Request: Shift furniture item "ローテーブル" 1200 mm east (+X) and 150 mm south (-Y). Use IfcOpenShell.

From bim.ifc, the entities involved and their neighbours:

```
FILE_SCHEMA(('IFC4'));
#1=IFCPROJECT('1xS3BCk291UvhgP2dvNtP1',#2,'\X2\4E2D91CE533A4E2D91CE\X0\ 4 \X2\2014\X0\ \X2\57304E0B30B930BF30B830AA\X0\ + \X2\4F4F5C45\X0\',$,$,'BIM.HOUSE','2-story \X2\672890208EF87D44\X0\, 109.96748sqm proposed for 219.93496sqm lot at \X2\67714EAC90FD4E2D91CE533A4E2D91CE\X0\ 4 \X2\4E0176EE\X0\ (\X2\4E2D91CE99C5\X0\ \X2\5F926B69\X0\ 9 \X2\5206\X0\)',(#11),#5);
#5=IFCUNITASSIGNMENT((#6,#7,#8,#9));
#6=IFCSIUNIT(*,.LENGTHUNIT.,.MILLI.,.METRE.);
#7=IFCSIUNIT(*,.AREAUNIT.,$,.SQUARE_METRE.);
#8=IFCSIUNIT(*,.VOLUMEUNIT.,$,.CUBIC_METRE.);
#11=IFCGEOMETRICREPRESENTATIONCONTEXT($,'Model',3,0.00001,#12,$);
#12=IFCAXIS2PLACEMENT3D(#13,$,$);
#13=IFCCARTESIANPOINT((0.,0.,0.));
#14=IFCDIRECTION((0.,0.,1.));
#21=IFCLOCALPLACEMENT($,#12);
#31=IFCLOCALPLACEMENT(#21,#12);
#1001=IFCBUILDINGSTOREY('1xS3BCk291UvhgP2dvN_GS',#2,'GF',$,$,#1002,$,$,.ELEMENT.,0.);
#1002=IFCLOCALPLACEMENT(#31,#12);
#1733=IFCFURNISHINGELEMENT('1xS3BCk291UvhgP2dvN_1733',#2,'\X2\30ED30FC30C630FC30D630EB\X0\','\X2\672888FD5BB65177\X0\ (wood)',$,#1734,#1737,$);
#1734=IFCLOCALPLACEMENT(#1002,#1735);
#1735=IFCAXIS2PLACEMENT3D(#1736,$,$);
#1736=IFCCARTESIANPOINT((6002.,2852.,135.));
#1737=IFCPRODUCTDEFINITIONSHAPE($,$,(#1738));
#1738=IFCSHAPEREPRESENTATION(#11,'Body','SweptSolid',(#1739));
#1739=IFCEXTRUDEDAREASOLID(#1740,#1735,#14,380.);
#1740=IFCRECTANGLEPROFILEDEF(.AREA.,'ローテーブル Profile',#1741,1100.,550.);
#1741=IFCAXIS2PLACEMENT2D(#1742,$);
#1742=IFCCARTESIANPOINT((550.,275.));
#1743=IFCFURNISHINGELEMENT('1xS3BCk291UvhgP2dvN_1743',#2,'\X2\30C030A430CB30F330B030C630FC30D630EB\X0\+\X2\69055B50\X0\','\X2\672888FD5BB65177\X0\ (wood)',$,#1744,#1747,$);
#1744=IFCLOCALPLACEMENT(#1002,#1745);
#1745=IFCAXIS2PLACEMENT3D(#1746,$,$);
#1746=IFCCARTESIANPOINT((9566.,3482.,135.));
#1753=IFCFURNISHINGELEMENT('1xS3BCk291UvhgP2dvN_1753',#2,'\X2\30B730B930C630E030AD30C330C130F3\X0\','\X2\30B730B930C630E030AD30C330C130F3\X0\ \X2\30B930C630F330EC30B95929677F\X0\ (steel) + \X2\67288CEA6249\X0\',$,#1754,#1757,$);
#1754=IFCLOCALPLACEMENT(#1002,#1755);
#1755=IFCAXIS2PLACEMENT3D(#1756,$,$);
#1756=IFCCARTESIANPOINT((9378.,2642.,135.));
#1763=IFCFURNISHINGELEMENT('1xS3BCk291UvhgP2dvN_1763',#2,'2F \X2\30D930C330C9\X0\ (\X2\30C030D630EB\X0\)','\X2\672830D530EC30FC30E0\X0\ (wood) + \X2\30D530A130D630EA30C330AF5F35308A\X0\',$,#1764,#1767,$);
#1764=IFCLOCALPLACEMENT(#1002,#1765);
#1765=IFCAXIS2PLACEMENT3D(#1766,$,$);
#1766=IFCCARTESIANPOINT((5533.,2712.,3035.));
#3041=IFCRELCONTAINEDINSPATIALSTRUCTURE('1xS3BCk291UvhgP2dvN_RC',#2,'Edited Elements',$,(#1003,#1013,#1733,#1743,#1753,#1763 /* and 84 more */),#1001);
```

```python
import ifcopenshell
import ifcopenshell.api.geometry
import ifcopenshell.util.placement
import ifcopenshell.util.unit

model = ifcopenshell.open("bim.ifc")
unit_scale = ifcopenshell.util.unit.calculate_unit_scale(model)

item = model.by_guid("1xS3BCk291UvhgP2dvN_1733")
matrix = ifcopenshell.util.placement.get_local_placement(item.ObjectPlacement)
matrix[0, 3] += 1.2 / unit_scale
matrix[1, 3] -= 0.15 / unit_scale
ifcopenshell.api.geometry.edit_object_placement(model, product=item, matrix=matrix, is_si=False)

print(ifcopenshell.util.placement.get_local_placement(item.ObjectPlacement).round(3) + 0.0)

model.write("bim_rev.ifc")
```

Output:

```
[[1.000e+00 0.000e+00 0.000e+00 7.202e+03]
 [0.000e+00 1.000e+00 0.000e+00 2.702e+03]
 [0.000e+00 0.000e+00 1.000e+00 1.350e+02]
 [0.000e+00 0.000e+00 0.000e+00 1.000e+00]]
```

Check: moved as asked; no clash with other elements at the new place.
